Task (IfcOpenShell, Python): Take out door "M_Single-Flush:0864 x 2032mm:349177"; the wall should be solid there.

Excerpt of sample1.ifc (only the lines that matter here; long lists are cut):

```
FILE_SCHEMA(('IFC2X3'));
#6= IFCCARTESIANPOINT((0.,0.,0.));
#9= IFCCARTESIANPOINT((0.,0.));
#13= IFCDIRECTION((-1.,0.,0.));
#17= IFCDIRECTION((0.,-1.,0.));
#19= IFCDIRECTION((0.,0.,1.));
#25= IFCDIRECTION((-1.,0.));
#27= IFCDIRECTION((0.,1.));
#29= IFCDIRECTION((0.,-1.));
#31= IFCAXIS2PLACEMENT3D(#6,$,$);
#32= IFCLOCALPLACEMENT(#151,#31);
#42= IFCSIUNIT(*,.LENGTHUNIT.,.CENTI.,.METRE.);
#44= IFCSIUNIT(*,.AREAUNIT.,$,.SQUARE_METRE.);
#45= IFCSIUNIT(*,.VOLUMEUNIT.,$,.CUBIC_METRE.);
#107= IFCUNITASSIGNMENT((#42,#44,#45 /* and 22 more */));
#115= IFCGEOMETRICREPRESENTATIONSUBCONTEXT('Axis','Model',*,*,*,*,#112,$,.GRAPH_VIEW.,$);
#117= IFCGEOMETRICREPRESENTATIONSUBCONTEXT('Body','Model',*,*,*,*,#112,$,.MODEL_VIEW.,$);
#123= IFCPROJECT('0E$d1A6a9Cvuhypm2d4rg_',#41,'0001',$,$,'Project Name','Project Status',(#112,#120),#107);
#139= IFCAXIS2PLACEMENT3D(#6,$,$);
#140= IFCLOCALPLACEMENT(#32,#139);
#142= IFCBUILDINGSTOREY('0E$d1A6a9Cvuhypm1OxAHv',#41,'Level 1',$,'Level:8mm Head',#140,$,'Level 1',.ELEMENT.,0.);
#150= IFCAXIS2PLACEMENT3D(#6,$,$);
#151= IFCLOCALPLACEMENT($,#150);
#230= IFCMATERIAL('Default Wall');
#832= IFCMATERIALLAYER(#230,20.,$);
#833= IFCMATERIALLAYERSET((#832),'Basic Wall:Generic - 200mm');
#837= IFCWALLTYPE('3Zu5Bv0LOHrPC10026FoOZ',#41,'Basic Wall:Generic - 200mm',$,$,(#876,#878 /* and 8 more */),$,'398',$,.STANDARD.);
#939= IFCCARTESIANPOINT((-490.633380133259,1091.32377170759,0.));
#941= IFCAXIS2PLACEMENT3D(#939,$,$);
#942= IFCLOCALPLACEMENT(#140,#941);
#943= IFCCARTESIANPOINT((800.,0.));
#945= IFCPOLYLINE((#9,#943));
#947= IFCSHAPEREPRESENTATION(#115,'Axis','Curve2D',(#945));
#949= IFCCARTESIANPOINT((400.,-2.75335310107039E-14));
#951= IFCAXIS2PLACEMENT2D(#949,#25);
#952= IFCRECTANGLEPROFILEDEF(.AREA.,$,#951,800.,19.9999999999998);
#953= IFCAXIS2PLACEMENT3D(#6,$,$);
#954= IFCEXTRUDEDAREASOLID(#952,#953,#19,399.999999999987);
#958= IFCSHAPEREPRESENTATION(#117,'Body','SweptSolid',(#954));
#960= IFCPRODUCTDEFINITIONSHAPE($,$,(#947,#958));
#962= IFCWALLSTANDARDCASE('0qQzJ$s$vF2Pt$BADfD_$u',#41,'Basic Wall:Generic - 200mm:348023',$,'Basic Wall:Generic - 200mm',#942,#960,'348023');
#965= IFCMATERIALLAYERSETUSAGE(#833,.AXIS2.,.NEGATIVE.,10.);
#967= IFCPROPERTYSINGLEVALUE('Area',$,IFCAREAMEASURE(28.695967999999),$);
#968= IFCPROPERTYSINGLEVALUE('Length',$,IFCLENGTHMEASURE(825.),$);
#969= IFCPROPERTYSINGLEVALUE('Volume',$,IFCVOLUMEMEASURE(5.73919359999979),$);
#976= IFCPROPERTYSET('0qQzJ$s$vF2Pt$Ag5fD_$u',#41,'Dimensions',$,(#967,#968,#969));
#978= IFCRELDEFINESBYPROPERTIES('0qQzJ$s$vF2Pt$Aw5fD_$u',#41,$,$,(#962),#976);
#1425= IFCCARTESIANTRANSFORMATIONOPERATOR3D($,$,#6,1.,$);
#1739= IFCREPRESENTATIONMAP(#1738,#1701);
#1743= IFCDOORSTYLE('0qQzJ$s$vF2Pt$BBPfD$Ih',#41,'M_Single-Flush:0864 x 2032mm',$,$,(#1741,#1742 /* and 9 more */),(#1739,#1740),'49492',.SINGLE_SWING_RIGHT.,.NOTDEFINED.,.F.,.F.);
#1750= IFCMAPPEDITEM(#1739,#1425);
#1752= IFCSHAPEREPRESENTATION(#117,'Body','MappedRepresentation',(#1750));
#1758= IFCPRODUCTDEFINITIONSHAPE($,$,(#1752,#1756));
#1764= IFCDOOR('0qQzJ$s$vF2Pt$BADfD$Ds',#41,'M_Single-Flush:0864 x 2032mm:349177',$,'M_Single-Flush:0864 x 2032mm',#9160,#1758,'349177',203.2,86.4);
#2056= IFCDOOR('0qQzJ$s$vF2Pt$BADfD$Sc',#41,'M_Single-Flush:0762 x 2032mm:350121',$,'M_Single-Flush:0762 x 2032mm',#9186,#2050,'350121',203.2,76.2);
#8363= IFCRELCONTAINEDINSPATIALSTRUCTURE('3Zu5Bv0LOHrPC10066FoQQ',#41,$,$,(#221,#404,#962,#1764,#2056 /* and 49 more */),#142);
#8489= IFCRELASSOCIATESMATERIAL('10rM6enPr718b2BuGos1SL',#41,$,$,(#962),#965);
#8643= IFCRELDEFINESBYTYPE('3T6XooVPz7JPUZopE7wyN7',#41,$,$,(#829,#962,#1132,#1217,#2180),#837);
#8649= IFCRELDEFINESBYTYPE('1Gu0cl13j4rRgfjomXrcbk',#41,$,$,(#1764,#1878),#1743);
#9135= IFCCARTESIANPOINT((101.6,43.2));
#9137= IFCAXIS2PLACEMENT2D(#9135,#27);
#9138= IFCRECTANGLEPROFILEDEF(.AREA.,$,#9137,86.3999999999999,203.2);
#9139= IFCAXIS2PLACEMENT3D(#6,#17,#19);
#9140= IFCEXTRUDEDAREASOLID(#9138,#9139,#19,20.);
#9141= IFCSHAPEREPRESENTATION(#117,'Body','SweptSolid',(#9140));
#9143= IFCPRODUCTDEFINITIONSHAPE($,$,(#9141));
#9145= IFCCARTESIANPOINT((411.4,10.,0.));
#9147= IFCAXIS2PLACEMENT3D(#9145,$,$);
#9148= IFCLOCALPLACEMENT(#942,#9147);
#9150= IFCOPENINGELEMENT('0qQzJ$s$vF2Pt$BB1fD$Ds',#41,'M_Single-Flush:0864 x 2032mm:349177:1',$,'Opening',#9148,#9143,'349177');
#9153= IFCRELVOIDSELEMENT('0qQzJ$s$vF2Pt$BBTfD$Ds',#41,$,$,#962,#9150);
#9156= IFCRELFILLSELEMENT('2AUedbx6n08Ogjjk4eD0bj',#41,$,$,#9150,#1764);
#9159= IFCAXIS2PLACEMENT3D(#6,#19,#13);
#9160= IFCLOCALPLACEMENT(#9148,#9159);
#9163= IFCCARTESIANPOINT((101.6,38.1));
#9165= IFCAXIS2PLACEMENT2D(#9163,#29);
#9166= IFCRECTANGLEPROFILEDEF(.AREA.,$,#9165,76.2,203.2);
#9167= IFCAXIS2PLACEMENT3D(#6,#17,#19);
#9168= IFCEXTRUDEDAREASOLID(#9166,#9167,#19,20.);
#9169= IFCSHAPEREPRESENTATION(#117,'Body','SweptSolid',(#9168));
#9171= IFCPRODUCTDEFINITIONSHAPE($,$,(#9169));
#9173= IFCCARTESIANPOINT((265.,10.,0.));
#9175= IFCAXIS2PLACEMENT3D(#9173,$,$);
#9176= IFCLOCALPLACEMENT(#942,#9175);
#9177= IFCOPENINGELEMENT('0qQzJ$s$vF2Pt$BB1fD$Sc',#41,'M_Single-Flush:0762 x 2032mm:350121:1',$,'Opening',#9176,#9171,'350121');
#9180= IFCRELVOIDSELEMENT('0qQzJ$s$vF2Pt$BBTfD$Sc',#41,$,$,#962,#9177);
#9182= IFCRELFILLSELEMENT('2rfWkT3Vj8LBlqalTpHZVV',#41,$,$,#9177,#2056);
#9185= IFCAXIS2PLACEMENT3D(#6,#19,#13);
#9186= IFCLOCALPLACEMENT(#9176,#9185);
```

```python
import ifcopenshell
import ifcopenshell.api.feature
import ifcopenshell.api.pset
import ifcopenshell.api.root
import ifcopenshell.geom
import ifcopenshell.util.element
import ifcopenshell.util.shape
import ifcopenshell.util.unit

model = ifcopenshell.open("sample1.ifc")
area_scale = ifcopenshell.util.unit.calculate_unit_scale(model, "AREAUNIT")
volume_scale = ifcopenshell.util.unit.calculate_unit_scale(model, "VOLUMEUNIT")
settings = ifcopenshell.geom.settings()


def volume(element):
    """Net volume in cubic metres, openings subtracted."""
    shape = ifcopenshell.geom.create_shape(settings, element)
    return ifcopenshell.util.shape.get_volume(shape.geometry)


door = model.by_id(1764)
opening = door.FillsVoids[0].RelatingOpeningElement
wall = opening.VoidsElements[0].RelatingBuildingElement
before = volume(wall)

ifcopenshell.api.root.remove_product(model, product=door)
ifcopenshell.api.feature.remove_feature(model, feature=opening)

after = volume(wall)
thickness = 0.2  # wall thickness in metres

# Update the wall's stored quantities.
pset = model.by_id(ifcopenshell.util.element.get_pset(wall, "Dimensions", should_inherit=False)["id"])
ifcopenshell.api.pset.edit_pset(model, pset=pset, properties={
    "Area": model.create_entity("IfcAreaMeasure", after / thickness / area_scale),
    "Volume": model.create_entity("IfcVolumeMeasure", after / volume_scale),
})

print(f"wall volume {before:.3f} -> {after:.3f} m3")

model.write("sample1_rev.ifc")
```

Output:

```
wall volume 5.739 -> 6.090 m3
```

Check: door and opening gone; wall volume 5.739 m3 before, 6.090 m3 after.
